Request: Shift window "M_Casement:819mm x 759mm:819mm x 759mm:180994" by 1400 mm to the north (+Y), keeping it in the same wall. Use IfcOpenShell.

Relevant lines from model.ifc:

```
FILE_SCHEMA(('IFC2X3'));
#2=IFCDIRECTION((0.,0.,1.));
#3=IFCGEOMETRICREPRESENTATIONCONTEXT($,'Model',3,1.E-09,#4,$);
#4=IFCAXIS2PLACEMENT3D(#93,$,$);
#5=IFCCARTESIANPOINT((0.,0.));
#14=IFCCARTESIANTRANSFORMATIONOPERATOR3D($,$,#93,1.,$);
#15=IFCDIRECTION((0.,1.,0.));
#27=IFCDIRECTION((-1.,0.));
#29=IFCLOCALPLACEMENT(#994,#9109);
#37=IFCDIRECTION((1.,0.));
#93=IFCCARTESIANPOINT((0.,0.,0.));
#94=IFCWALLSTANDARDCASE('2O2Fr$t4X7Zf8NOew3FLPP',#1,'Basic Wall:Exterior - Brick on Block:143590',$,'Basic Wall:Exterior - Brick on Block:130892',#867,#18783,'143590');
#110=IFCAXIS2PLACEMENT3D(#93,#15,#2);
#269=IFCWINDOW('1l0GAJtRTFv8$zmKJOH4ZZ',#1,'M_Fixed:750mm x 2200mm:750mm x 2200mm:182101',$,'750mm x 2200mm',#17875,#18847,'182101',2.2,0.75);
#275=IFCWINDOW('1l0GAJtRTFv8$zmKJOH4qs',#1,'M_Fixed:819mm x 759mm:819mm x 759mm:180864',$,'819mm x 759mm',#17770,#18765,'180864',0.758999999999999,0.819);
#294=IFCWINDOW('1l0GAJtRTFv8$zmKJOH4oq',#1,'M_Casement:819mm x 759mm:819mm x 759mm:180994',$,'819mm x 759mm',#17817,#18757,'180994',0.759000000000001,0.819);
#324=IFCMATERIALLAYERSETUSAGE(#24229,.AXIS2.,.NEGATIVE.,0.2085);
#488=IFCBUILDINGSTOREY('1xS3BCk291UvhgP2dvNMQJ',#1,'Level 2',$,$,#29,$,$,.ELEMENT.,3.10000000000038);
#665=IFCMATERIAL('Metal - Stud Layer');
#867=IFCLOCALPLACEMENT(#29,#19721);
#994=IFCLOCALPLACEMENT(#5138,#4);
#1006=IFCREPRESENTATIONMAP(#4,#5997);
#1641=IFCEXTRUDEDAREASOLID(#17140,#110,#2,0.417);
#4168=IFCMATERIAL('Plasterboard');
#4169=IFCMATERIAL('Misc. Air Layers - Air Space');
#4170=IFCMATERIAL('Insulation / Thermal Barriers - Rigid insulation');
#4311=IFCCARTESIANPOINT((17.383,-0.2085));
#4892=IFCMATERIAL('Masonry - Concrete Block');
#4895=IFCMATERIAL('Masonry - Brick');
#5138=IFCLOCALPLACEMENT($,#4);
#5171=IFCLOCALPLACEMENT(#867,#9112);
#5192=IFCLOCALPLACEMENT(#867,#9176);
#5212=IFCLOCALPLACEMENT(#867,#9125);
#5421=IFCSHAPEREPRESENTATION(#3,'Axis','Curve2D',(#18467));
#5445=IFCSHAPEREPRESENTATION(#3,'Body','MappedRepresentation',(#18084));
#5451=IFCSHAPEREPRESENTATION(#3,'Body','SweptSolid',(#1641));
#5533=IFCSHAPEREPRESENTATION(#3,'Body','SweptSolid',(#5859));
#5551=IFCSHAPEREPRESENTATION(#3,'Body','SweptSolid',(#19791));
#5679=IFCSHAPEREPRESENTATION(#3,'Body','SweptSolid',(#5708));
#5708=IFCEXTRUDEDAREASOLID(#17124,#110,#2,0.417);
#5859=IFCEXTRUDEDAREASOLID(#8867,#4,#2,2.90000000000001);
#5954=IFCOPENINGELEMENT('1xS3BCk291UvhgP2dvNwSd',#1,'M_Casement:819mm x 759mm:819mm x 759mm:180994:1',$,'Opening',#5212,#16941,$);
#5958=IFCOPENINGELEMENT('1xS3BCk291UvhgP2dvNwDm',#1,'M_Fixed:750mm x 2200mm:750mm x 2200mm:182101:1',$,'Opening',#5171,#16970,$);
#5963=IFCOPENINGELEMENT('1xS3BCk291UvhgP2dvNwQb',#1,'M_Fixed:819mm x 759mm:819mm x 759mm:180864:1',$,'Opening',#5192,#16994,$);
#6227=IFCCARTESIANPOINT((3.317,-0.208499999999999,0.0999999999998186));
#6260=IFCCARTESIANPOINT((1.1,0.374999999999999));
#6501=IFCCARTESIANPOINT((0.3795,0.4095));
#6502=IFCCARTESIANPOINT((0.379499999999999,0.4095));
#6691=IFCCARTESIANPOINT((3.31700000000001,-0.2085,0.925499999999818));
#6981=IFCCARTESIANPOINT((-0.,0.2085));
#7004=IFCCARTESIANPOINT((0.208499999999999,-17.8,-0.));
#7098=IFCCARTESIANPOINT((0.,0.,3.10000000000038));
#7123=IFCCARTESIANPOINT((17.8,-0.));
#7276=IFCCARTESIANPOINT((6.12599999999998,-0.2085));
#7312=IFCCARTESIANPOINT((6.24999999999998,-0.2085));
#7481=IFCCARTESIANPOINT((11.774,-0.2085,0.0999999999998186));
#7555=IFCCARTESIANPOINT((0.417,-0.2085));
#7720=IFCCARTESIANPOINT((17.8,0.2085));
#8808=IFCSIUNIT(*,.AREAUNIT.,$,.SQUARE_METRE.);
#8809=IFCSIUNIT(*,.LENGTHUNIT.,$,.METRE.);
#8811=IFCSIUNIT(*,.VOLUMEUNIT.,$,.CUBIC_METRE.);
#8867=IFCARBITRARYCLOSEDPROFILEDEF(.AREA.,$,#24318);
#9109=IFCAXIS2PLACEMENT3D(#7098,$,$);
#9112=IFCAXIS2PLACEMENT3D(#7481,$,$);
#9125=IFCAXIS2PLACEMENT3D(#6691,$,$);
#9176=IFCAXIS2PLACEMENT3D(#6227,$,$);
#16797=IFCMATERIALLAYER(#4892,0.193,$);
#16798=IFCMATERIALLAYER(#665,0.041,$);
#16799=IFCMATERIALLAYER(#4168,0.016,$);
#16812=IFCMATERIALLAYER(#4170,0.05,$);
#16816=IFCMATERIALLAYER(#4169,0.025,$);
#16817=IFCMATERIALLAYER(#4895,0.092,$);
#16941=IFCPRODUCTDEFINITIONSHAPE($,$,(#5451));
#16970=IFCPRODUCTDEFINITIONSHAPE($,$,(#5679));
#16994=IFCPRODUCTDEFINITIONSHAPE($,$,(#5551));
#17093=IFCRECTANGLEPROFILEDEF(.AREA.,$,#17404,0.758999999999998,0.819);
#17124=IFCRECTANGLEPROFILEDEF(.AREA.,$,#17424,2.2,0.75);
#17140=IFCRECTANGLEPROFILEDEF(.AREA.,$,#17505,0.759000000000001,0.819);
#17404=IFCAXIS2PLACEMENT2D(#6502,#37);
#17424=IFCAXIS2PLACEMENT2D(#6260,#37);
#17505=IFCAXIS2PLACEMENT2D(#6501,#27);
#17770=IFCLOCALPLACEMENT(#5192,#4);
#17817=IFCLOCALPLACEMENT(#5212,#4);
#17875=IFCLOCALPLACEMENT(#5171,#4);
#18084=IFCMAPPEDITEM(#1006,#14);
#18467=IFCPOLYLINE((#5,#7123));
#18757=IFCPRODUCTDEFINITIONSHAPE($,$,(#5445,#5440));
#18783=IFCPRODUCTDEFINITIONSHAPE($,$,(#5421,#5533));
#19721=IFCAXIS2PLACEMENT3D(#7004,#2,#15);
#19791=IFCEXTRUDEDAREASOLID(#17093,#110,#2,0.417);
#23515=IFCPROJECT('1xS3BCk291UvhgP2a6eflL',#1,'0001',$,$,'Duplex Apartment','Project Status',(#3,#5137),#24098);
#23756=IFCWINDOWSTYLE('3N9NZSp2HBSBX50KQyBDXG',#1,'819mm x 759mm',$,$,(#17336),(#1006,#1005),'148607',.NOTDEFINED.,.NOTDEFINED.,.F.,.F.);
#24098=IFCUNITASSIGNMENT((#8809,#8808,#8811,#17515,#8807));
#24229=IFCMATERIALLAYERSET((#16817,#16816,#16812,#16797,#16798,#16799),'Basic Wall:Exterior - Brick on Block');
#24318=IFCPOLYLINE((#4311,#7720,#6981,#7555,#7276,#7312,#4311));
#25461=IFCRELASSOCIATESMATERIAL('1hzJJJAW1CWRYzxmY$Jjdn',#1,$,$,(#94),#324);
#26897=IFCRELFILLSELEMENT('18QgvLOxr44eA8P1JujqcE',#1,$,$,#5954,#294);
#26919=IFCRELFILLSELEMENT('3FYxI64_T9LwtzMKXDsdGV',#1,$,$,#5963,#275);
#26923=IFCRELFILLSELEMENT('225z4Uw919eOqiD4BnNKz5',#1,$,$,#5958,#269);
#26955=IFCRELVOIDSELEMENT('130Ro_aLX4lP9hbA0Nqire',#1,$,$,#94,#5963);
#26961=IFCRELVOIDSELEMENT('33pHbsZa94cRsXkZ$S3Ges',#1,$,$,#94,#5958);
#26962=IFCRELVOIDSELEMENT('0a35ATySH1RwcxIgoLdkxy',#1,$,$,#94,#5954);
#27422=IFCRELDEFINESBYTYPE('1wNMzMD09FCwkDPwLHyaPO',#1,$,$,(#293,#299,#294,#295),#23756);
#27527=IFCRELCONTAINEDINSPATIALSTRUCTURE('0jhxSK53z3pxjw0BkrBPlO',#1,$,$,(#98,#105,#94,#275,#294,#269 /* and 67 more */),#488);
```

```python
import ifcopenshell
import ifcopenshell.api.geometry
import ifcopenshell.util.placement
import ifcopenshell.util.unit

model = ifcopenshell.open("model.ifc")
unit_scale = ifcopenshell.util.unit.calculate_unit_scale(model)

window = model.by_id(294)
opening = window.FillsVoids[0].RelatingOpeningElement
wall = opening.VoidsElements[0].RelatingBuildingElement

wall_matrix = ifcopenshell.util.placement.get_local_placement(wall.ObjectPlacement)
shift = wall_matrix[:3, 0] * 1.4 / unit_scale
before = ifcopenshell.util.placement.get_local_placement(window.ObjectPlacement)[:3, 3].copy()

# The window is placed relative to its opening, so it follows when the opening moves.
matrix = ifcopenshell.util.placement.get_local_placement(opening.ObjectPlacement)
matrix[:3, 3] += shift
ifcopenshell.api.geometry.edit_object_placement(
    model, product=opening, matrix=matrix, is_si=False, should_transform_children=True
)

after = ifcopenshell.util.placement.get_local_placement(window.ObjectPlacement)[:3, 3]
print("window moved by", (after - before).round(3) + 0.0)

model.write("model_updated.ifc")
```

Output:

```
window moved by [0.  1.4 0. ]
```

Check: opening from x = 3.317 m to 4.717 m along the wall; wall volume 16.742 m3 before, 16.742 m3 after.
